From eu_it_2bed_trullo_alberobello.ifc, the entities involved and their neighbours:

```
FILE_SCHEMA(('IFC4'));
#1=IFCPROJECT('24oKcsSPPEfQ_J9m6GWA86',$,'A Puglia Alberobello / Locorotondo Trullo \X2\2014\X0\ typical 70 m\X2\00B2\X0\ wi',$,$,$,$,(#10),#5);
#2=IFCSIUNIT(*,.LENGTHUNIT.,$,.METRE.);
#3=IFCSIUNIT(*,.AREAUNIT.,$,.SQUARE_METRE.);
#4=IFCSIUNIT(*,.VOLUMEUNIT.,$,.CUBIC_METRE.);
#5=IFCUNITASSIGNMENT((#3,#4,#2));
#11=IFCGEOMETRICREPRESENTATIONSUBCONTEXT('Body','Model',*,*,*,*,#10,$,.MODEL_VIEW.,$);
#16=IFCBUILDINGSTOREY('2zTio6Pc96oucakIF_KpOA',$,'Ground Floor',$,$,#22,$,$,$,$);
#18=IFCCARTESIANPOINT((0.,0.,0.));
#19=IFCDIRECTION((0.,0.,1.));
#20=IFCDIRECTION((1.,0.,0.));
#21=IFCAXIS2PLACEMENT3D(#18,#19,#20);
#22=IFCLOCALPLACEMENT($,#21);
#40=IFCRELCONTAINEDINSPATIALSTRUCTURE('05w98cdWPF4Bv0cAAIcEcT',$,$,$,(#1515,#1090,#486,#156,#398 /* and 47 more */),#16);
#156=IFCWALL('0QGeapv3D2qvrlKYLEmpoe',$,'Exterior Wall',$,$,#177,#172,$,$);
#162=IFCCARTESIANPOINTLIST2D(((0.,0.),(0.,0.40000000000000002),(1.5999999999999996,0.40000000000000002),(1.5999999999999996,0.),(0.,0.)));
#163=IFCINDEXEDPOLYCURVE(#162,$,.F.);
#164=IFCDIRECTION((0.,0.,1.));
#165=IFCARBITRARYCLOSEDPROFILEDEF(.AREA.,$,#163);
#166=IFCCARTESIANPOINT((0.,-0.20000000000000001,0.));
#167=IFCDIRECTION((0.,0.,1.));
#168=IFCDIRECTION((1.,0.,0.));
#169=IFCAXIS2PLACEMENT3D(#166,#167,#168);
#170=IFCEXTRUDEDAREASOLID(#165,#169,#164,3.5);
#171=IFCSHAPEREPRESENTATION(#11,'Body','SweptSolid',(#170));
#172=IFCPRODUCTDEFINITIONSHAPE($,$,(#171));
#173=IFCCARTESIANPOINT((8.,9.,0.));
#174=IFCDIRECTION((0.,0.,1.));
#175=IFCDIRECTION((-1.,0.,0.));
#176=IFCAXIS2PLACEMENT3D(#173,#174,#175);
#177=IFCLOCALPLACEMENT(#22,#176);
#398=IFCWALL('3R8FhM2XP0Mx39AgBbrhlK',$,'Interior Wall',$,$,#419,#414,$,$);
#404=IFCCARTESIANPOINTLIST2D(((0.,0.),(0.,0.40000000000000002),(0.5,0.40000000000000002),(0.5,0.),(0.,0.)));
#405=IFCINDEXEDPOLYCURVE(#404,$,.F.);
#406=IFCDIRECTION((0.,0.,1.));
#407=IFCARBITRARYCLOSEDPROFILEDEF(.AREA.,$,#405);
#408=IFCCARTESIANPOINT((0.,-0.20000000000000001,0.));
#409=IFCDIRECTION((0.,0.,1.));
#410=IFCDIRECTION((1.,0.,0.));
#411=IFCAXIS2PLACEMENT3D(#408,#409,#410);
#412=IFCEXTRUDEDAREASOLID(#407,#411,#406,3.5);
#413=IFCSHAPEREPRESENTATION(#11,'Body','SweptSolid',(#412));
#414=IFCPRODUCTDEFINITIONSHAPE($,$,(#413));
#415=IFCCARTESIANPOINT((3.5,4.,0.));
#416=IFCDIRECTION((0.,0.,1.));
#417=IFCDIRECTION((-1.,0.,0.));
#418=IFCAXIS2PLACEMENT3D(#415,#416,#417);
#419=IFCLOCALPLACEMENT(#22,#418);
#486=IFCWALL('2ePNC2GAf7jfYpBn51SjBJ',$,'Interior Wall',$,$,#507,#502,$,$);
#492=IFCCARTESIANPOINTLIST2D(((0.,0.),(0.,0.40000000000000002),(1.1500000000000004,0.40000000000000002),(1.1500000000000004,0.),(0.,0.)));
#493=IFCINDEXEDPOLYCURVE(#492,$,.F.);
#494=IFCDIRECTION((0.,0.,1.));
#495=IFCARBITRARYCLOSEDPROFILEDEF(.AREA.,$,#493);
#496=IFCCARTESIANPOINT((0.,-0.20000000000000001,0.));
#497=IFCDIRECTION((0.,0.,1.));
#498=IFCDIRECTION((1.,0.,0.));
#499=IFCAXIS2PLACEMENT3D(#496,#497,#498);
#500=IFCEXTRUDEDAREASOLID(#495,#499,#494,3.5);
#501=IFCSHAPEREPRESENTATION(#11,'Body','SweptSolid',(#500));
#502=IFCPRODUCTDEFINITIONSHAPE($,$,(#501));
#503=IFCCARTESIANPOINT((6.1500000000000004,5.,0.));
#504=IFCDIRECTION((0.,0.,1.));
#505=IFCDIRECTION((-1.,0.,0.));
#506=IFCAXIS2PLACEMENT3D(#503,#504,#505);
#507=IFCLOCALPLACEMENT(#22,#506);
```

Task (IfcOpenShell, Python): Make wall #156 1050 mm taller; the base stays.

```python
import ifcopenshell
import ifcopenshell.geom
import ifcopenshell.util.representation
import ifcopenshell.util.shape
import ifcopenshell.util.unit

model = ifcopenshell.open("eu_it_2bed_trullo_alberobello.ifc")
unit_scale = ifcopenshell.util.unit.calculate_unit_scale(model)
settings = ifcopenshell.geom.settings()


def volume(element):
    """Net volume in cubic metres, openings subtracted."""
    shape = ifcopenshell.geom.create_shape(settings, element)
    return ifcopenshell.util.shape.get_volume(shape.geometry)


wall = model.by_guid("0QGeapv3D2qvrlKYLEmpoe")
before = volume(wall)

body = ifcopenshell.util.representation.get_representation(wall, "Model", "Body")
solid = body.Items[0]
old_height = solid.Depth
solid.Depth += 1.05 / unit_scale
after = volume(wall)

print(f"height {old_height:g} -> {solid.Depth:g}, volume {before:.3f} -> {after:.3f} m3")

model.write("eu_it_2bed_trullo_alberobello_rev.ifc")
```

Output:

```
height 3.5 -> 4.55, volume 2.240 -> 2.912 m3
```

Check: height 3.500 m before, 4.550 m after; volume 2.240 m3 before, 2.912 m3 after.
